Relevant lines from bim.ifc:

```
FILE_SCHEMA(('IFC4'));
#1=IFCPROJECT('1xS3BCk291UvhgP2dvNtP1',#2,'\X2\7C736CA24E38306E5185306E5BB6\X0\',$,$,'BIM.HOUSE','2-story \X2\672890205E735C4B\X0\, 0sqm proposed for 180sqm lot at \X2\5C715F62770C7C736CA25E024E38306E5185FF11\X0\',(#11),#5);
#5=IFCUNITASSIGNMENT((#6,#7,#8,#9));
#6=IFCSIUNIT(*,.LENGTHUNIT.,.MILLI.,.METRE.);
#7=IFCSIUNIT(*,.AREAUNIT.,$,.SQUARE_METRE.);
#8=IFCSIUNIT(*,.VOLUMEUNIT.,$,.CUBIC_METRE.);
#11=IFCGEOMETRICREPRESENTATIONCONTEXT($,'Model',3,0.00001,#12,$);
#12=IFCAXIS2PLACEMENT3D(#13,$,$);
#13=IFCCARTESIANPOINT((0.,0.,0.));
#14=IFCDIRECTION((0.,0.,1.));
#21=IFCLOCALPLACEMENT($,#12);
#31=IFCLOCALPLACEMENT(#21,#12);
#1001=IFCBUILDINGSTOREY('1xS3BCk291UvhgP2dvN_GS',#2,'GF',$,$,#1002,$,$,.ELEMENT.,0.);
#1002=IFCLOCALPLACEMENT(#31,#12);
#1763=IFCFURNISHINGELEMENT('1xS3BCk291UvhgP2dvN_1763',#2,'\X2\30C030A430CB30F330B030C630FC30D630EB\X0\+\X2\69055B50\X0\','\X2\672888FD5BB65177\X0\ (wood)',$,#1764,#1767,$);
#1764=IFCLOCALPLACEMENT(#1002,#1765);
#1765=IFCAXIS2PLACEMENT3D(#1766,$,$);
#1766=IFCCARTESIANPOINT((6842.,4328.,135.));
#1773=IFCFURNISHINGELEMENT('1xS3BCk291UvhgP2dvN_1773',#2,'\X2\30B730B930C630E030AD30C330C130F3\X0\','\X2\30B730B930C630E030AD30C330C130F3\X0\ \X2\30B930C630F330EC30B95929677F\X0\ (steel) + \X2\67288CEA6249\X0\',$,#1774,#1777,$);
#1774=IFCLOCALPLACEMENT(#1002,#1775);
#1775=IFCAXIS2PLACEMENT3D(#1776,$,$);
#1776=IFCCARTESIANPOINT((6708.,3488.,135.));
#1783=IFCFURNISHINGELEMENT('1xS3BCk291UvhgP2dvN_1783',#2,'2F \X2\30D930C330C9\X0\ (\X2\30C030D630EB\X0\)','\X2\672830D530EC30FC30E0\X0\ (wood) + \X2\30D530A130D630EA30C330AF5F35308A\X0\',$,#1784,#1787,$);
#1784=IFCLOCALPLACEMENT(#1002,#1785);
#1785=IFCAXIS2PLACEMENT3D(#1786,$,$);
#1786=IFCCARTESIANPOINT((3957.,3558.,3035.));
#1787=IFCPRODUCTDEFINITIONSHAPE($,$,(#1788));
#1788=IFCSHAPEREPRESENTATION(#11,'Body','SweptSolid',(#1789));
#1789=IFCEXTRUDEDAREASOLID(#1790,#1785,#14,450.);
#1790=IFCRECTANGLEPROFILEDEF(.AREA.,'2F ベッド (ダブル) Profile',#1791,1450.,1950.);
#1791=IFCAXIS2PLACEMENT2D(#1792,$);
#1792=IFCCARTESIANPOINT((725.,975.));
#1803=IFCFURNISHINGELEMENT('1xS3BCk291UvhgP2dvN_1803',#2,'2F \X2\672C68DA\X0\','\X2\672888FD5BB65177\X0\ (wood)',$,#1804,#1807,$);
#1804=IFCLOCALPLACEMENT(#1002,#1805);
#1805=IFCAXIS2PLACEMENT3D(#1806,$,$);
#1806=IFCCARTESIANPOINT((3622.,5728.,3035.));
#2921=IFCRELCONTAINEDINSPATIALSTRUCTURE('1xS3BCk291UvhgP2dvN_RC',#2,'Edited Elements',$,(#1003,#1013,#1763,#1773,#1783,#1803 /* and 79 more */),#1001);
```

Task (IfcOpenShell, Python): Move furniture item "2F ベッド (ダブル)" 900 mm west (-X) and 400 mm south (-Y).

```python
import ifcopenshell
import ifcopenshell.api.geometry
import ifcopenshell.util.placement

model = ifcopenshell.open("bim.ifc")

item = model.by_guid("1xS3BCk291UvhgP2dvN_1783")
matrix = ifcopenshell.util.placement.get_local_placement(item.ObjectPlacement)
matrix[0, 3] -= 900.0
matrix[1, 3] -= 400.0
ifcopenshell.api.geometry.edit_object_placement(model, product=item, matrix=matrix, is_si=False)

print(ifcopenshell.util.placement.get_local_placement(item.ObjectPlacement).round(3) + 0.0)

model.write("bim-out.ifc")
```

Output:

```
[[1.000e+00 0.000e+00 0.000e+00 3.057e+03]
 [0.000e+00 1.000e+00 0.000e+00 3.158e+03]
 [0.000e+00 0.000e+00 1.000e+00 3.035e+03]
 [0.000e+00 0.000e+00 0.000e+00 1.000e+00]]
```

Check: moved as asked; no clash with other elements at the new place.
